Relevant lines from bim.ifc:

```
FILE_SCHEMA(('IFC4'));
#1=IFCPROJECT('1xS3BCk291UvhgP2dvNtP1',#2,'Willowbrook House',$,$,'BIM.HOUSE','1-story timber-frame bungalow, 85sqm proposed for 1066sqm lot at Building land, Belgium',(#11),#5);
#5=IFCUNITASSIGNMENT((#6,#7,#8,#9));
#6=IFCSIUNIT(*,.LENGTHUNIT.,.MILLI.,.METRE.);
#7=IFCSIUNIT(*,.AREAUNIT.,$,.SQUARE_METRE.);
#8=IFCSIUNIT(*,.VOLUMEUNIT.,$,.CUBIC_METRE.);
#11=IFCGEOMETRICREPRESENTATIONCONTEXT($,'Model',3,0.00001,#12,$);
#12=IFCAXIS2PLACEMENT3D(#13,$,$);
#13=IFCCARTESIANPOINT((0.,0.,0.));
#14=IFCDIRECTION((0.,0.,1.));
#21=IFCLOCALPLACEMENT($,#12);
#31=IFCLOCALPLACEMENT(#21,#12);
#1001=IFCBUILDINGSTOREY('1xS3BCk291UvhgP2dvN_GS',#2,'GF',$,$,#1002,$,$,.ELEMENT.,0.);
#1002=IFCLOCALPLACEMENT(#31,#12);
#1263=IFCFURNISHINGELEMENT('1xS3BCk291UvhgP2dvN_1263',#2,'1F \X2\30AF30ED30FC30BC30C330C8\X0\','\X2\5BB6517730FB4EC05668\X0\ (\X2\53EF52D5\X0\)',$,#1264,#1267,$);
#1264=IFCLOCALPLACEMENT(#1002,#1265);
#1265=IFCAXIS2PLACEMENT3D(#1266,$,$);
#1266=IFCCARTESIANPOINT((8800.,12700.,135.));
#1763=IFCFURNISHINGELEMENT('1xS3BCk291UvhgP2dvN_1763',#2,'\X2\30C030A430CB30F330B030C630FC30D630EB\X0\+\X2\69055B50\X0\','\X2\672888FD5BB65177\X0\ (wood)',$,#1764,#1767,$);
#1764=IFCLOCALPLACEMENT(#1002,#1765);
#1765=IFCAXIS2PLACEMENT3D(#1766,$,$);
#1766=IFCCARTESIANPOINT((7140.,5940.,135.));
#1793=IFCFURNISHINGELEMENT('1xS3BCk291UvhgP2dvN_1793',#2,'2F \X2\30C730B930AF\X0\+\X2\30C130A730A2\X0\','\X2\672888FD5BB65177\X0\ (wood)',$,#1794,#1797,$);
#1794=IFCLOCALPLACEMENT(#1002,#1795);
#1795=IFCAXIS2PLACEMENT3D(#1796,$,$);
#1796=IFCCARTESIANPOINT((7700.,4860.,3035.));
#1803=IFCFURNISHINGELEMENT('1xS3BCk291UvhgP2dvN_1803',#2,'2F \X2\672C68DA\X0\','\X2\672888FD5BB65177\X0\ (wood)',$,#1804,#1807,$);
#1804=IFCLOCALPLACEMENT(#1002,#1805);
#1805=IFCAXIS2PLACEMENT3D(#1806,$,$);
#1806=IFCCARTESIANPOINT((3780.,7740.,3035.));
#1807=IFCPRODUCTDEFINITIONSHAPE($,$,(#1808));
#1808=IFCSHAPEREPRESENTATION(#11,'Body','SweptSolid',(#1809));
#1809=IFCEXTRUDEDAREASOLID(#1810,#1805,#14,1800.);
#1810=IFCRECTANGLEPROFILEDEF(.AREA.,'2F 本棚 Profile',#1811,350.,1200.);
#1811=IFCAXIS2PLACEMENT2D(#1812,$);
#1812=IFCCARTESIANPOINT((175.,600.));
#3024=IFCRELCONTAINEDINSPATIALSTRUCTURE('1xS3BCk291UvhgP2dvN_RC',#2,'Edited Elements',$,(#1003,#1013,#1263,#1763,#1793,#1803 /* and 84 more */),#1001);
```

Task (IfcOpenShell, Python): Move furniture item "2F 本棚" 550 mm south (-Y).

```python
import ifcopenshell
import ifcopenshell.api.geometry
import ifcopenshell.util.placement

model = ifcopenshell.open("bim.ifc")

item = model.by_guid("1xS3BCk291UvhgP2dvN_1803")
matrix = ifcopenshell.util.placement.get_local_placement(item.ObjectPlacement)
matrix[1, 3] -= 550.0
ifcopenshell.api.geometry.edit_object_placement(model, product=item, matrix=matrix, is_si=False)

print(ifcopenshell.util.placement.get_local_placement(item.ObjectPlacement).round(3) + 0.0)

model.write("bim_v2.ifc")
```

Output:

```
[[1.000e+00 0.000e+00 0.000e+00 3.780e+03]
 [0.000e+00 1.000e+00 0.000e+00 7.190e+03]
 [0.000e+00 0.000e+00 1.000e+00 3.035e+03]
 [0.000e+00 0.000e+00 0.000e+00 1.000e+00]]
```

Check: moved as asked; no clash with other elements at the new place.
